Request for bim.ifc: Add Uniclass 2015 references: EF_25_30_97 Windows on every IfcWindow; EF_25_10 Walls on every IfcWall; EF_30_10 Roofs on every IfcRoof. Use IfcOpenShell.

First a look at what the model holds.

```python
import ifcopenshell

model = ifcopenshell.open("bim.ifc")
print(model.schema)
print("classifications:", [c.Name for c in model.by_type("IfcClassification")])
for ifc_class in ("IfcDoor", "IfcRoof", "IfcStair", "IfcWall", "IfcWindow"):
    print(ifc_class, len(model.by_type(ifc_class)))
```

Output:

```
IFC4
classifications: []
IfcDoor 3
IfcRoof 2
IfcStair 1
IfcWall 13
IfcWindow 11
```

```python
import ifcopenshell
import ifcopenshell.api.classification

model = ifcopenshell.open("bim.ifc")

system = ifcopenshell.api.classification.add_classification(model, classification="Uniclass 2015")

codes = {
    "IfcWindow": ("EF_25_30_97", "Windows"),
    "IfcWall": ("EF_25_10", "Walls"),
    "IfcRoof": ("EF_30_10", "Roofs"),
}
for ifc_class, (code, name) in codes.items():
    products = model.by_type(ifc_class)
    ifcopenshell.api.classification.add_reference(
        model, products=products, classification=system, identification=code, name=name
    )
    print(code, len(products))

model.write("bim_updated.ifc")
```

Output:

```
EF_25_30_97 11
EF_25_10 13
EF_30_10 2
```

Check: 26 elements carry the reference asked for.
